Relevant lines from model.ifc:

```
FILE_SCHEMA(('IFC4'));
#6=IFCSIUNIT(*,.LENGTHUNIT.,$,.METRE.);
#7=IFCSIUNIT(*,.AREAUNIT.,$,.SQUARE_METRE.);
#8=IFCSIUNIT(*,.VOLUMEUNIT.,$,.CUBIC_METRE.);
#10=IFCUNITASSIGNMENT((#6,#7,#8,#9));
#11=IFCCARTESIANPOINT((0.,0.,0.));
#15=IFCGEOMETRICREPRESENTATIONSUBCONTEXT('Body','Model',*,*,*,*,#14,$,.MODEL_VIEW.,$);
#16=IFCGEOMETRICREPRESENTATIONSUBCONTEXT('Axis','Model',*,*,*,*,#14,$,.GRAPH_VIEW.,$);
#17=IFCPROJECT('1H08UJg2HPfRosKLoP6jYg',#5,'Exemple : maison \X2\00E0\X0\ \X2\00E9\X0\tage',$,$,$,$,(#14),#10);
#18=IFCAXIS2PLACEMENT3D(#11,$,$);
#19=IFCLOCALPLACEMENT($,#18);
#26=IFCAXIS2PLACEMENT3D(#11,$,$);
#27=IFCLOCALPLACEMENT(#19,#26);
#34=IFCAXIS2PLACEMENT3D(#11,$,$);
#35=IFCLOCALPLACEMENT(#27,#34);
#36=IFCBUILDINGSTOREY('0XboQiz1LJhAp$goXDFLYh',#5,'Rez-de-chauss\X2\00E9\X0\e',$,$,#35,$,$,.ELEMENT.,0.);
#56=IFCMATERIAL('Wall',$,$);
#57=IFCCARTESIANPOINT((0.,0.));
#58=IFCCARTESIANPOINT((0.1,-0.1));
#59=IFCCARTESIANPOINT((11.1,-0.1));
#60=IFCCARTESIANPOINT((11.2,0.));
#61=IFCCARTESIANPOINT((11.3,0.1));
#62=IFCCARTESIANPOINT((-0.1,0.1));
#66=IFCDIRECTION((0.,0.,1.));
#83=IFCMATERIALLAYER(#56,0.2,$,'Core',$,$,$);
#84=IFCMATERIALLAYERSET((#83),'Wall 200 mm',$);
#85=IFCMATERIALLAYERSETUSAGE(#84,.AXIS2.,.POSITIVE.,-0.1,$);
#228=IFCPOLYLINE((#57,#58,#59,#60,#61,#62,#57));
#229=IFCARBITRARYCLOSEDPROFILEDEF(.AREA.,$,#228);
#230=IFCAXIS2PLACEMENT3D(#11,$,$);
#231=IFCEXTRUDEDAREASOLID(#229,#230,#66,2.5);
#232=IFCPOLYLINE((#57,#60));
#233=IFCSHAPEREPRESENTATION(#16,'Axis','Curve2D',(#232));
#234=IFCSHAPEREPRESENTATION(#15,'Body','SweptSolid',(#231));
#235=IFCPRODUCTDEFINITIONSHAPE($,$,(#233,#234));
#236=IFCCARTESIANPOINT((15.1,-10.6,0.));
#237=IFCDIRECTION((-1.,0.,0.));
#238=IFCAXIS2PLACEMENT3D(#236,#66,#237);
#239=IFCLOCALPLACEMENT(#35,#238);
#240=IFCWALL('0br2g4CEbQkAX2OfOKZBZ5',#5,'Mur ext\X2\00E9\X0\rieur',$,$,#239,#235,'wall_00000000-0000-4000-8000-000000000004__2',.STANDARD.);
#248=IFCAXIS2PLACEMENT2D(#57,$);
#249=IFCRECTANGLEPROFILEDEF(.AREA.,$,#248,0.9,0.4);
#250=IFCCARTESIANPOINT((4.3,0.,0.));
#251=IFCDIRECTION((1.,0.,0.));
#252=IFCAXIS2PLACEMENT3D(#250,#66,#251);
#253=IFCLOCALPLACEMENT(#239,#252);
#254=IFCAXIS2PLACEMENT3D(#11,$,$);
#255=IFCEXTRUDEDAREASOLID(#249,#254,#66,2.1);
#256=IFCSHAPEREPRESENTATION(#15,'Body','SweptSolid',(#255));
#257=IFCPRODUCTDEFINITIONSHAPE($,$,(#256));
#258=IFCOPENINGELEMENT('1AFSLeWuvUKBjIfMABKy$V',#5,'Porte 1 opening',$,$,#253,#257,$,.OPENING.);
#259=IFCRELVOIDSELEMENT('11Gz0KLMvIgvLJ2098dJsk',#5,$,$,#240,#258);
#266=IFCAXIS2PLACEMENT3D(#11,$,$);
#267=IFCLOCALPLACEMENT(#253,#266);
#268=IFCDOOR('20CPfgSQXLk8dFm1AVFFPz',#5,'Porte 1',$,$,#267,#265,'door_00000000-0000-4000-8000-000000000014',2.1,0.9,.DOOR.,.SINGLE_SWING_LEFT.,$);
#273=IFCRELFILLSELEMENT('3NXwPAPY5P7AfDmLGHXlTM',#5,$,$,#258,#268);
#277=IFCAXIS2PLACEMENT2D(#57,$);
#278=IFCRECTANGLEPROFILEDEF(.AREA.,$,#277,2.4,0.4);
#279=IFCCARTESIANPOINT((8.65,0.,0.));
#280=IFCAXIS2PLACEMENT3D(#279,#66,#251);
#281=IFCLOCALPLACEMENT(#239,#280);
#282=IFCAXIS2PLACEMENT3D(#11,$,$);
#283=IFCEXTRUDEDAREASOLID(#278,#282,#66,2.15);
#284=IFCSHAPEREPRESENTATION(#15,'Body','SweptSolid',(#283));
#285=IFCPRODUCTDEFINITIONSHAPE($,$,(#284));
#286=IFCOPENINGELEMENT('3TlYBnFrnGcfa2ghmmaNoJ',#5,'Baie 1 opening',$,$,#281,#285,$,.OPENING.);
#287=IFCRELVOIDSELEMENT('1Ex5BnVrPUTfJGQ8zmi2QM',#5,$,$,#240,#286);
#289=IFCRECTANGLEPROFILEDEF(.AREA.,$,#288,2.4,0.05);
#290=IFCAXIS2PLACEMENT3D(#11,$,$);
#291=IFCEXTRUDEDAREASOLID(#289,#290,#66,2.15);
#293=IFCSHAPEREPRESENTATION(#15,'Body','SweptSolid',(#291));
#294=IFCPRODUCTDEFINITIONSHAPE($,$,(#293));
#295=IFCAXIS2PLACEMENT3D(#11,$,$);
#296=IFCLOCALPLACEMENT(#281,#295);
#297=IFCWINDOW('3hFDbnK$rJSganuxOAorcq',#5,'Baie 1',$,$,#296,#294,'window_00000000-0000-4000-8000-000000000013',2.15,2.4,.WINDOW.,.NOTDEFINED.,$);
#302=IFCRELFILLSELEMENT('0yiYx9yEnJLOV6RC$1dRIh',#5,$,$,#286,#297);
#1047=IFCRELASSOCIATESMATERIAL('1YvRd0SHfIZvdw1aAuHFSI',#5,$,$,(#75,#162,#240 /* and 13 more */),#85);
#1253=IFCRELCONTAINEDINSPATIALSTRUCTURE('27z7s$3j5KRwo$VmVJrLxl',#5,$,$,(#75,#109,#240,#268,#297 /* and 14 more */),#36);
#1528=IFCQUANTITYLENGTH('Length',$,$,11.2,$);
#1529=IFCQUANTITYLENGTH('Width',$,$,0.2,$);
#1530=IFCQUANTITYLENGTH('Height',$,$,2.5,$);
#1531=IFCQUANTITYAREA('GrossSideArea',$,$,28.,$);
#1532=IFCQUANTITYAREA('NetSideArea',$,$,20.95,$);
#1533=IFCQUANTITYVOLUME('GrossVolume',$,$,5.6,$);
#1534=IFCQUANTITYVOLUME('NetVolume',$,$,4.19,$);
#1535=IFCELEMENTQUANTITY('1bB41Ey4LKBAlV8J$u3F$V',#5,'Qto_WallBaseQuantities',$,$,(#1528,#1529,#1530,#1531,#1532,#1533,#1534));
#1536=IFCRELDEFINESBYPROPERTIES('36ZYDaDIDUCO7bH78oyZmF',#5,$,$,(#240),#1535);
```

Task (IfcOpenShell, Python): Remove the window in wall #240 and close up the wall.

```python
import ifcopenshell
import ifcopenshell.api.feature
import ifcopenshell.api.pset
import ifcopenshell.api.root
import ifcopenshell.geom
import ifcopenshell.util.element
import ifcopenshell.util.shape
import ifcopenshell.util.unit

model = ifcopenshell.open("model.ifc")
area_scale = ifcopenshell.util.unit.calculate_unit_scale(model, "AREAUNIT")
volume_scale = ifcopenshell.util.unit.calculate_unit_scale(model, "VOLUMEUNIT")
settings = ifcopenshell.geom.settings()


def volume(element):
    """Net volume in cubic metres, openings subtracted."""
    shape = ifcopenshell.geom.create_shape(settings, element)
    return ifcopenshell.util.shape.get_volume(shape.geometry)


window = model.by_guid("3hFDbnK$rJSganuxOAorcq")
opening = window.FillsVoids[0].RelatingOpeningElement
wall = opening.VoidsElements[0].RelatingBuildingElement
before = volume(wall)

ifcopenshell.api.root.remove_product(model, product=window)
ifcopenshell.api.feature.remove_feature(model, feature=opening)

after = volume(wall)
thickness = 0.2  # wall thickness in metres

# Update the wall's stored quantities.
qto = model.by_id(ifcopenshell.util.element.get_pset(wall, "Qto_WallBaseQuantities", should_inherit=False)["id"])
ifcopenshell.api.pset.edit_qto(model, qto=qto, properties={
    "NetSideArea": after / thickness / area_scale,
    "NetVolume": after / volume_scale,
})

print(f"wall volume {before:.3f} -> {after:.3f} m3")

model.write("model-out.ifc")
```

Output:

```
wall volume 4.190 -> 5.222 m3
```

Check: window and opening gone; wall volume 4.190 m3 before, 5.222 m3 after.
